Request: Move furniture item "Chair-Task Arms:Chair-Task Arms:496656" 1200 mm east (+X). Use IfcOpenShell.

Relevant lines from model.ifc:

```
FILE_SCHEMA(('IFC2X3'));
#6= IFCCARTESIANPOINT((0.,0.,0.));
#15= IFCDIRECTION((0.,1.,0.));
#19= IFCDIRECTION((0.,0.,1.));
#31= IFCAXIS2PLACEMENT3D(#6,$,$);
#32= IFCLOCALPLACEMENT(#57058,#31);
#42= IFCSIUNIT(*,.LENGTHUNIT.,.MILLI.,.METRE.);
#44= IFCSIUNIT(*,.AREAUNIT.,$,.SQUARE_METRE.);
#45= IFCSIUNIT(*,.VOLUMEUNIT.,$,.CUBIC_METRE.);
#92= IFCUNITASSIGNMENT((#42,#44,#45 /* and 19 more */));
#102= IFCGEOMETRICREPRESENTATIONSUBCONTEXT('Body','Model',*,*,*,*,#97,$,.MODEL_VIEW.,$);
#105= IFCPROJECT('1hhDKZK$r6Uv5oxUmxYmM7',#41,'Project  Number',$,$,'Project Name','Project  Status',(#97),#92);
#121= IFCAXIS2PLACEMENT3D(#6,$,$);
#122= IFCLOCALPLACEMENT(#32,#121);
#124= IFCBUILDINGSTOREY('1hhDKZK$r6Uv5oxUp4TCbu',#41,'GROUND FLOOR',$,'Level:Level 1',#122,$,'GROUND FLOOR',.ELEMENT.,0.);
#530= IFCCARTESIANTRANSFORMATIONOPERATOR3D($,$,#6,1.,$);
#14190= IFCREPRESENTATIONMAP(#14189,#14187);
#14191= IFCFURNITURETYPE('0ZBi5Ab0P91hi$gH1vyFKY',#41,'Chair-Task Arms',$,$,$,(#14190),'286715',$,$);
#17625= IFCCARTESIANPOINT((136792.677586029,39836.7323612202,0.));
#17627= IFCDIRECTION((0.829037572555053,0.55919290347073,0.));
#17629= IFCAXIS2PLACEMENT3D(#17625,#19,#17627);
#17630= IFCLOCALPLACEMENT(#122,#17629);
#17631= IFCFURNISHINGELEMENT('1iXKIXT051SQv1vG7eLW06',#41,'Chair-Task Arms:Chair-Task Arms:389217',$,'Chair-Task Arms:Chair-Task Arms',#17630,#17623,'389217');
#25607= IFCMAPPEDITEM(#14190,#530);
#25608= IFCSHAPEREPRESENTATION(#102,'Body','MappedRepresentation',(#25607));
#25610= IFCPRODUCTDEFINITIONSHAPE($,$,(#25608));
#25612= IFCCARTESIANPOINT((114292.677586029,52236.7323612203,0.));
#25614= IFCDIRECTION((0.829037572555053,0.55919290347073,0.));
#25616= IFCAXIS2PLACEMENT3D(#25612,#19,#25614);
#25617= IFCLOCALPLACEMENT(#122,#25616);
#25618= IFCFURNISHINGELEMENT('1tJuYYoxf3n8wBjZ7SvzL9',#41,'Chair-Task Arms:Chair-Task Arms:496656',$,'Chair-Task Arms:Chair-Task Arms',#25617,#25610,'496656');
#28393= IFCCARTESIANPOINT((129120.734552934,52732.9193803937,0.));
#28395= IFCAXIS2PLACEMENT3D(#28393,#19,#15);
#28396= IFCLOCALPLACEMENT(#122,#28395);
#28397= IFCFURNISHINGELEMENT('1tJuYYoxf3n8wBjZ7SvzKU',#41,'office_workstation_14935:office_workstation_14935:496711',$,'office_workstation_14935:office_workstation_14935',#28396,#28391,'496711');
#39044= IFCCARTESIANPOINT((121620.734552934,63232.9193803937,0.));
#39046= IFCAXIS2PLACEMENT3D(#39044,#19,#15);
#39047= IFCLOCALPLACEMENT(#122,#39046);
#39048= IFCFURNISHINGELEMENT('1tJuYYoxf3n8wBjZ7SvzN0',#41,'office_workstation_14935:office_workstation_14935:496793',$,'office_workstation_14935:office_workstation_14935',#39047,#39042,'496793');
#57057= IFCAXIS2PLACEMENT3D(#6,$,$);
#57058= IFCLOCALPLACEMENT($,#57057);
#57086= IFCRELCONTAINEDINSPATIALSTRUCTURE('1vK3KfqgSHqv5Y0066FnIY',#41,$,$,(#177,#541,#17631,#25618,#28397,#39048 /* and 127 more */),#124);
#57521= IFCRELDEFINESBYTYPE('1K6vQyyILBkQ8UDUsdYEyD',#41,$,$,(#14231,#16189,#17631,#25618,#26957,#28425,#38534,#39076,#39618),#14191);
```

```python
import ifcopenshell
import ifcopenshell.api.geometry
import ifcopenshell.util.placement

model = ifcopenshell.open("model.ifc")

item = model.by_id(25618)
matrix = ifcopenshell.util.placement.get_local_placement(item.ObjectPlacement)
matrix[0, 3] += 1200.0
ifcopenshell.api.geometry.edit_object_placement(model, product=item, matrix=matrix, is_si=False)

print(ifcopenshell.util.placement.get_local_placement(item.ObjectPlacement).round(3) + 0.0)

model.write("model_v2.ifc")
```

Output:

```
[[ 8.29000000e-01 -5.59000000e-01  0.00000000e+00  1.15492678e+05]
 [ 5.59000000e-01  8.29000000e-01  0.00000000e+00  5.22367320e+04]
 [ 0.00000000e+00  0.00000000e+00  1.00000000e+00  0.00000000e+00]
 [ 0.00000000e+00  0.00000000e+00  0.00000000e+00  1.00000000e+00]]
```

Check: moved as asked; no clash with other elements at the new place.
